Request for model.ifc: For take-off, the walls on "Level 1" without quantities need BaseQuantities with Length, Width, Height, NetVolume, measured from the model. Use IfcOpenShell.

First a look at what the model holds.

```python
import ifcopenshell
import ifcopenshell.util.element
import ifcopenshell.util.unit

model = ifcopenshell.open("model.ifc")
print(model.schema)
for unit_type in ("LENGTHUNIT", "AREAUNIT", "VOLUMEUNIT"):
    print(unit_type, ifcopenshell.util.unit.calculate_unit_scale(model, unit_type))
storey = next(s for s in model.by_type("IfcBuildingStorey") if s.Name == "Level 1")
walls = [e for e in ifcopenshell.util.element.get_decomposition(storey) if e.is_a("IfcWall")]
for e in sorted(walls, key=lambda e: e.id()):
    print(e.id(), e.is_a(), e.Name, list(ifcopenshell.util.element.get_psets(e, qtos_only=True)), sep=" | ")
```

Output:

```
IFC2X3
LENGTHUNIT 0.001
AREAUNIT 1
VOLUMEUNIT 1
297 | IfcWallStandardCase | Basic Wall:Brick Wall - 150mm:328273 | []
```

```python
import ifcopenshell
import ifcopenshell.api.pset
import ifcopenshell.geom
import ifcopenshell.util.element
import ifcopenshell.util.shape
import ifcopenshell.util.unit

model = ifcopenshell.open("model.ifc")
unit_scale = ifcopenshell.util.unit.calculate_unit_scale(model)
volume_scale = ifcopenshell.util.unit.calculate_unit_scale(model, "VOLUMEUNIT")
settings = ifcopenshell.geom.settings()

storey = next(s for s in model.by_type("IfcBuildingStorey") if s.Name == "Level 1")
walls = [e for e in ifcopenshell.util.element.get_decomposition(storey) if e.is_a("IfcWall")]

for e in sorted(walls, key=lambda e: e.id()):
    if ifcopenshell.util.element.get_psets(e, qtos_only=True, should_inherit=False):
        continue
    # Geometry comes back in metres, in the element's own axes.
    shape = ifcopenshell.geom.create_shape(settings, e)
    values = {
        "Length": ifcopenshell.util.shape.get_x(shape.geometry) / unit_scale,
        "Width": ifcopenshell.util.shape.get_y(shape.geometry) / unit_scale,
        "Height": ifcopenshell.util.shape.get_z(shape.geometry) / unit_scale,
        "NetVolume": ifcopenshell.util.shape.get_volume(shape.geometry) / volume_scale,
    }
    qto = ifcopenshell.api.pset.add_qto(model, product=e, name="BaseQuantities")
    ifcopenshell.api.pset.edit_qto(model, qto=qto, properties=values)
    print(e.id(), {k: round(v, 3) for k, v in values.items()})

model.write("model_rev.ifc")
```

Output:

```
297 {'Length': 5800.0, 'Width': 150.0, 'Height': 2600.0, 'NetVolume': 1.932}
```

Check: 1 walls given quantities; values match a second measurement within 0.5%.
